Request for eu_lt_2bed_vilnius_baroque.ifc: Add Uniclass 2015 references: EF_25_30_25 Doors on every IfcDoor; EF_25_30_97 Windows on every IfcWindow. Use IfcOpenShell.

First a look at what the model holds.

```python
import ifcopenshell

model = ifcopenshell.open("eu_lt_2bed_vilnius_baroque.ifc")
print(model.schema)
print("classifications:", [c.Name for c in model.by_type("IfcClassification")])
for ifc_class in ("IfcDoor", "IfcRoof", "IfcStair", "IfcWall", "IfcWindow"):
    print(ifc_class, len(model.by_type(ifc_class)))
```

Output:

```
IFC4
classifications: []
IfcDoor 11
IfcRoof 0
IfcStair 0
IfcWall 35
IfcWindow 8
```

```python
import ifcopenshell
import ifcopenshell.api.classification

model = ifcopenshell.open("eu_lt_2bed_vilnius_baroque.ifc")

system = ifcopenshell.api.classification.add_classification(model, classification="Uniclass 2015")

codes = {
    "IfcDoor": ("EF_25_30_25", "Doors"),
    "IfcWindow": ("EF_25_30_97", "Windows"),
}
for ifc_class, (code, name) in codes.items():
    products = model.by_type(ifc_class)
    ifcopenshell.api.classification.add_reference(
        model, products=products, classification=system, identification=code, name=name
    )
    print(code, len(products))

model.write("eu_lt_2bed_vilnius_baroque_v2.ifc")
```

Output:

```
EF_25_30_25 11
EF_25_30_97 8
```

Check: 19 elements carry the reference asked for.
